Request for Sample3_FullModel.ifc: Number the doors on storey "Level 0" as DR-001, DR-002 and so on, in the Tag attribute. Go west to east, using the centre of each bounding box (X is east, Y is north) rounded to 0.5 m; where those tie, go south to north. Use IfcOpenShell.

First a look at what the model holds.

```python
import ifcopenshell
import ifcopenshell.util.element
import ifcopenshell.util.placement

model = ifcopenshell.open("Sample3_FullModel.ifc")
print(model.schema)
storey = next(s for s in model.by_type("IfcBuildingStorey") if s.Name == "Level 0")
doors = [e for e in ifcopenshell.util.element.get_decomposition(storey) if e.is_a("IfcDoor")]
for e in sorted(doors, key=lambda e: e.id()):
    origin = ifcopenshell.util.placement.get_local_placement(e.ObjectPlacement)[:3, 3]
    print(e.id(), e.Tag, e.Name, origin.round(2) + 0.0, sep=" | ")
```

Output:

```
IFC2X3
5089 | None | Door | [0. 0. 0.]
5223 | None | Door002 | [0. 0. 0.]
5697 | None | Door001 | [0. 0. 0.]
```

```python
import ifcopenshell
import ifcopenshell.geom
import ifcopenshell.util.element
import ifcopenshell.util.shape

model = ifcopenshell.open("Sample3_FullModel.ifc")
settings = ifcopenshell.geom.settings()
settings.set("use-world-coords", True)


def centre(element):
    shape = ifcopenshell.geom.create_shape(settings, element)
    return ifcopenshell.util.shape.get_bbox_centroid(shape.geometry)


storey = next(s for s in model.by_type("IfcBuildingStorey") if s.Name == "Level 0")
doors = [e for e in ifcopenshell.util.element.get_decomposition(storey) if e.is_a("IfcDoor")]

# Insertion points can sit at a corner or the storey origin, so sort by the geometry (in metres).
centres = {e: centre(e) for e in doors}
doors.sort(key=lambda e: (round(centres[e][0] / 0.5), centres[e][1]))

for i, e in enumerate(doors, start=1):
    number = f"DR-0{i:02d}"
    e.Tag = number
    print(e.id(), number)

model.write("Sample3_FullModel-out.ifc")
```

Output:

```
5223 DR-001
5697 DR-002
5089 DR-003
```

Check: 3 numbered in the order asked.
